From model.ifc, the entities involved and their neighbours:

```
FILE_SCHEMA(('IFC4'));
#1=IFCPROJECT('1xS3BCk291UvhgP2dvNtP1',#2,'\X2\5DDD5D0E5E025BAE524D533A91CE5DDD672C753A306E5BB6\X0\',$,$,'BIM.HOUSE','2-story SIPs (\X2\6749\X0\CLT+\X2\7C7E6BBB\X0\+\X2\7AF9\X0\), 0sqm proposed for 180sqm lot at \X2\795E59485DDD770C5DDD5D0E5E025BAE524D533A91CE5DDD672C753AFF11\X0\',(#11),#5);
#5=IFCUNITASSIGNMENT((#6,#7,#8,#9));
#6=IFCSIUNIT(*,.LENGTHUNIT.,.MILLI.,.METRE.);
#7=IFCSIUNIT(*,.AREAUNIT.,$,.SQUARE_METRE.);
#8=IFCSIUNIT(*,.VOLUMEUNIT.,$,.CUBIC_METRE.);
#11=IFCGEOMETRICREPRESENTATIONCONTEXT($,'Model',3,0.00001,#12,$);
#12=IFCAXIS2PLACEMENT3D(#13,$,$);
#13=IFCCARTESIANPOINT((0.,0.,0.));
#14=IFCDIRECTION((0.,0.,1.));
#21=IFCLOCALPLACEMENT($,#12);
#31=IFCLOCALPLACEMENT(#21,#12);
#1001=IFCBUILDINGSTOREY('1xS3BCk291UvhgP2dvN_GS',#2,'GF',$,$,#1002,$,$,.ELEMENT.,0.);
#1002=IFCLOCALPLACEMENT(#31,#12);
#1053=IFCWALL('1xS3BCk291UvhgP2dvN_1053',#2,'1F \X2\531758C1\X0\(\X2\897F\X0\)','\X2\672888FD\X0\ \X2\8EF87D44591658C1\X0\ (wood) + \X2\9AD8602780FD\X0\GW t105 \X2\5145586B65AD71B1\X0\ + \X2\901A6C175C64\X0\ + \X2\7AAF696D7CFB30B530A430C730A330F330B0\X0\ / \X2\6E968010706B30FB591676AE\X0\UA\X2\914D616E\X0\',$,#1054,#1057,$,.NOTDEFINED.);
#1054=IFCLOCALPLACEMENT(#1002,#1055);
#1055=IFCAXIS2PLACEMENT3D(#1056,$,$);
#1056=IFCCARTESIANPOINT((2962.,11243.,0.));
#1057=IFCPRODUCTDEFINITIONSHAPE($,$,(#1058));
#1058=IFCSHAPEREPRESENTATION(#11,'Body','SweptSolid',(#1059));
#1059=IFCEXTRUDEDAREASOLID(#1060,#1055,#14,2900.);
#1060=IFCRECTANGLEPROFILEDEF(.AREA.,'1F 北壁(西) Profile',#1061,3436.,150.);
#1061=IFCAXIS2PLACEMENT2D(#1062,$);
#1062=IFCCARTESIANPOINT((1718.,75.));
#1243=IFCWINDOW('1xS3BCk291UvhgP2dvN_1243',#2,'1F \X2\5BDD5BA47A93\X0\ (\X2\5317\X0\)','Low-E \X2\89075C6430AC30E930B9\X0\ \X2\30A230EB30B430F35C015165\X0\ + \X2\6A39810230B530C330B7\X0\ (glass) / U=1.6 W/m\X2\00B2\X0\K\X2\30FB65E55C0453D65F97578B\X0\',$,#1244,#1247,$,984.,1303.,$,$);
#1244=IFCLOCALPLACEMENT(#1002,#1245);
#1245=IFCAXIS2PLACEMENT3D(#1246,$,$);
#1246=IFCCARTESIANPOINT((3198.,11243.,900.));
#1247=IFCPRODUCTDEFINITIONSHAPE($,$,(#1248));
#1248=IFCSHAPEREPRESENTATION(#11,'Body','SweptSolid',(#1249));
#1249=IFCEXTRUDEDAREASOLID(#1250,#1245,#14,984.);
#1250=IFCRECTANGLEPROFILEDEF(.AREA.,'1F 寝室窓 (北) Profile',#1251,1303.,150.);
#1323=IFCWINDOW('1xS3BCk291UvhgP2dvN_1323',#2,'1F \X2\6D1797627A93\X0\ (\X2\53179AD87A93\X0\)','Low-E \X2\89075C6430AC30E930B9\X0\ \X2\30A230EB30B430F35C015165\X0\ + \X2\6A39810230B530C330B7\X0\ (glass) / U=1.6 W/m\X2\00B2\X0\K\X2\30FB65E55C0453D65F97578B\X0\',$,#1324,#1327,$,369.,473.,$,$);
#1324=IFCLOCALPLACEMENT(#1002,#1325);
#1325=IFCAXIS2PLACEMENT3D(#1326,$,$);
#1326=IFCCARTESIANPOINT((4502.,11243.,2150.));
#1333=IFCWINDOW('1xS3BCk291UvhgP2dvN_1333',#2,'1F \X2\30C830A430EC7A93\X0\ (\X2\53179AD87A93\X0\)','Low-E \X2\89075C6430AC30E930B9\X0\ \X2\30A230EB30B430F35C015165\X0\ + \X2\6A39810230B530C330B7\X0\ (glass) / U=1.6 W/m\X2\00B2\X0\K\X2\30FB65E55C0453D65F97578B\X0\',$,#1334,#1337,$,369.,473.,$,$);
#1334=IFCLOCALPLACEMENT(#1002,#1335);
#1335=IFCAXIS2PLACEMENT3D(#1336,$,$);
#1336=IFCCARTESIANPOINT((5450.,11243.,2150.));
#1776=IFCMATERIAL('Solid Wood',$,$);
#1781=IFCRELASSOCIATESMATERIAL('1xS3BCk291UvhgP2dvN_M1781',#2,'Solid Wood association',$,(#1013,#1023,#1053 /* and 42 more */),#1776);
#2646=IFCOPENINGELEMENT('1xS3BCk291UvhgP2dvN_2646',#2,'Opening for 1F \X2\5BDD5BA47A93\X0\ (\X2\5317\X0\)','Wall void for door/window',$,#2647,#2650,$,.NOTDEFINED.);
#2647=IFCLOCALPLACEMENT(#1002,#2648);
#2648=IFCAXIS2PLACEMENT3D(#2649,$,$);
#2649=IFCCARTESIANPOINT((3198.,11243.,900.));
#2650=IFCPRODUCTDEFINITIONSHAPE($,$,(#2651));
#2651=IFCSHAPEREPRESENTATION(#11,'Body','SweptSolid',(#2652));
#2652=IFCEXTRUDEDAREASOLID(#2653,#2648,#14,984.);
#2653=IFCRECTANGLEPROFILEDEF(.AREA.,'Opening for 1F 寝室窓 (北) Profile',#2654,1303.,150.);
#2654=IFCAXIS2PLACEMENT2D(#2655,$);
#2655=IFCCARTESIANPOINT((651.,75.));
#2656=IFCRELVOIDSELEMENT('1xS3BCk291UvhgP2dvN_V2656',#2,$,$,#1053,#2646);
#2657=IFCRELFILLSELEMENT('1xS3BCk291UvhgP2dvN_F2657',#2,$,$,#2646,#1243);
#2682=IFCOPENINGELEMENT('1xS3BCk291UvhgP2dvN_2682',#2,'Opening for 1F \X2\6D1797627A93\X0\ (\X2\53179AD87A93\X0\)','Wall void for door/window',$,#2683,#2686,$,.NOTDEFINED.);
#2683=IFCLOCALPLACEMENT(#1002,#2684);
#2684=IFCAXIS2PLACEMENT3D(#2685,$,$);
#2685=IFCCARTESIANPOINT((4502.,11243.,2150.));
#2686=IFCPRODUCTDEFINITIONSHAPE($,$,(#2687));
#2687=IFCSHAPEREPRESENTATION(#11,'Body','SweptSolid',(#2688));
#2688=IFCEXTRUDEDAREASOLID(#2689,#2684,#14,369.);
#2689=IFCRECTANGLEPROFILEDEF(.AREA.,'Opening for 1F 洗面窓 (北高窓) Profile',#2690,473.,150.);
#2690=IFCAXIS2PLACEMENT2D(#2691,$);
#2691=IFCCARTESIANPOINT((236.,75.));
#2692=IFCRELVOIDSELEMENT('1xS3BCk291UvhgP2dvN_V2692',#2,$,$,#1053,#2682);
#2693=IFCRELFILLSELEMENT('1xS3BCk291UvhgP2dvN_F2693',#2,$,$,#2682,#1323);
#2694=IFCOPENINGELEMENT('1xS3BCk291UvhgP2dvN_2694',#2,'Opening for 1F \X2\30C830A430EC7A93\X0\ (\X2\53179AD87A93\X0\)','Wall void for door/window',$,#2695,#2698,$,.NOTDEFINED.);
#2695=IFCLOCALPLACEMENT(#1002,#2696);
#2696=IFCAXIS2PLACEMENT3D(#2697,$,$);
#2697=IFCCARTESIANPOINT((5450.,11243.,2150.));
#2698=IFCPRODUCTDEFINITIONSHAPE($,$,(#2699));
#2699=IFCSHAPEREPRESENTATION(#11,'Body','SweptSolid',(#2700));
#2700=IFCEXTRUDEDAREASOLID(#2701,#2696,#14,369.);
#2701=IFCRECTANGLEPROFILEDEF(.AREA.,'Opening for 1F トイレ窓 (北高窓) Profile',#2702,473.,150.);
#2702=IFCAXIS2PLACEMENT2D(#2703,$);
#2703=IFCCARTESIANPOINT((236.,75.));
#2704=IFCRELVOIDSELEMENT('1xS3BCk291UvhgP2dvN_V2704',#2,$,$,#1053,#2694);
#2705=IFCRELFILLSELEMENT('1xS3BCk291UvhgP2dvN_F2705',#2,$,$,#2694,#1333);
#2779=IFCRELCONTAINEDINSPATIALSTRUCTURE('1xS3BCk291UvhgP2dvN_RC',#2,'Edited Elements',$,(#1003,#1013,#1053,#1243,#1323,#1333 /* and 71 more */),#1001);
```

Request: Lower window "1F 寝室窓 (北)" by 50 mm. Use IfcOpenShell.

```python
import numpy as np
import ifcopenshell
import ifcopenshell.api.geometry
import ifcopenshell.util.placement
import ifcopenshell.util.unit

model = ifcopenshell.open("model.ifc")
unit_scale = ifcopenshell.util.unit.calculate_unit_scale(model)

window = model.by_guid("1xS3BCk291UvhgP2dvN_1243")
opening = window.FillsVoids[0].RelatingOpeningElement
dz = -50.0

shift = np.array([0.0, 0.0, dz])
# The window is not placed relative to its opening, so move both.
for product in (opening, window):
    matrix = ifcopenshell.util.placement.get_local_placement(product.ObjectPlacement)
    matrix[:3, 3] += shift
    ifcopenshell.api.geometry.edit_object_placement(model, product=product, matrix=matrix, is_si=False)

print(f"moved by {dz * unit_scale:+.3f} m")

model.write("model_rev.ifc")
```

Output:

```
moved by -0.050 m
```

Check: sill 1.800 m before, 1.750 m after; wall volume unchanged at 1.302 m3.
